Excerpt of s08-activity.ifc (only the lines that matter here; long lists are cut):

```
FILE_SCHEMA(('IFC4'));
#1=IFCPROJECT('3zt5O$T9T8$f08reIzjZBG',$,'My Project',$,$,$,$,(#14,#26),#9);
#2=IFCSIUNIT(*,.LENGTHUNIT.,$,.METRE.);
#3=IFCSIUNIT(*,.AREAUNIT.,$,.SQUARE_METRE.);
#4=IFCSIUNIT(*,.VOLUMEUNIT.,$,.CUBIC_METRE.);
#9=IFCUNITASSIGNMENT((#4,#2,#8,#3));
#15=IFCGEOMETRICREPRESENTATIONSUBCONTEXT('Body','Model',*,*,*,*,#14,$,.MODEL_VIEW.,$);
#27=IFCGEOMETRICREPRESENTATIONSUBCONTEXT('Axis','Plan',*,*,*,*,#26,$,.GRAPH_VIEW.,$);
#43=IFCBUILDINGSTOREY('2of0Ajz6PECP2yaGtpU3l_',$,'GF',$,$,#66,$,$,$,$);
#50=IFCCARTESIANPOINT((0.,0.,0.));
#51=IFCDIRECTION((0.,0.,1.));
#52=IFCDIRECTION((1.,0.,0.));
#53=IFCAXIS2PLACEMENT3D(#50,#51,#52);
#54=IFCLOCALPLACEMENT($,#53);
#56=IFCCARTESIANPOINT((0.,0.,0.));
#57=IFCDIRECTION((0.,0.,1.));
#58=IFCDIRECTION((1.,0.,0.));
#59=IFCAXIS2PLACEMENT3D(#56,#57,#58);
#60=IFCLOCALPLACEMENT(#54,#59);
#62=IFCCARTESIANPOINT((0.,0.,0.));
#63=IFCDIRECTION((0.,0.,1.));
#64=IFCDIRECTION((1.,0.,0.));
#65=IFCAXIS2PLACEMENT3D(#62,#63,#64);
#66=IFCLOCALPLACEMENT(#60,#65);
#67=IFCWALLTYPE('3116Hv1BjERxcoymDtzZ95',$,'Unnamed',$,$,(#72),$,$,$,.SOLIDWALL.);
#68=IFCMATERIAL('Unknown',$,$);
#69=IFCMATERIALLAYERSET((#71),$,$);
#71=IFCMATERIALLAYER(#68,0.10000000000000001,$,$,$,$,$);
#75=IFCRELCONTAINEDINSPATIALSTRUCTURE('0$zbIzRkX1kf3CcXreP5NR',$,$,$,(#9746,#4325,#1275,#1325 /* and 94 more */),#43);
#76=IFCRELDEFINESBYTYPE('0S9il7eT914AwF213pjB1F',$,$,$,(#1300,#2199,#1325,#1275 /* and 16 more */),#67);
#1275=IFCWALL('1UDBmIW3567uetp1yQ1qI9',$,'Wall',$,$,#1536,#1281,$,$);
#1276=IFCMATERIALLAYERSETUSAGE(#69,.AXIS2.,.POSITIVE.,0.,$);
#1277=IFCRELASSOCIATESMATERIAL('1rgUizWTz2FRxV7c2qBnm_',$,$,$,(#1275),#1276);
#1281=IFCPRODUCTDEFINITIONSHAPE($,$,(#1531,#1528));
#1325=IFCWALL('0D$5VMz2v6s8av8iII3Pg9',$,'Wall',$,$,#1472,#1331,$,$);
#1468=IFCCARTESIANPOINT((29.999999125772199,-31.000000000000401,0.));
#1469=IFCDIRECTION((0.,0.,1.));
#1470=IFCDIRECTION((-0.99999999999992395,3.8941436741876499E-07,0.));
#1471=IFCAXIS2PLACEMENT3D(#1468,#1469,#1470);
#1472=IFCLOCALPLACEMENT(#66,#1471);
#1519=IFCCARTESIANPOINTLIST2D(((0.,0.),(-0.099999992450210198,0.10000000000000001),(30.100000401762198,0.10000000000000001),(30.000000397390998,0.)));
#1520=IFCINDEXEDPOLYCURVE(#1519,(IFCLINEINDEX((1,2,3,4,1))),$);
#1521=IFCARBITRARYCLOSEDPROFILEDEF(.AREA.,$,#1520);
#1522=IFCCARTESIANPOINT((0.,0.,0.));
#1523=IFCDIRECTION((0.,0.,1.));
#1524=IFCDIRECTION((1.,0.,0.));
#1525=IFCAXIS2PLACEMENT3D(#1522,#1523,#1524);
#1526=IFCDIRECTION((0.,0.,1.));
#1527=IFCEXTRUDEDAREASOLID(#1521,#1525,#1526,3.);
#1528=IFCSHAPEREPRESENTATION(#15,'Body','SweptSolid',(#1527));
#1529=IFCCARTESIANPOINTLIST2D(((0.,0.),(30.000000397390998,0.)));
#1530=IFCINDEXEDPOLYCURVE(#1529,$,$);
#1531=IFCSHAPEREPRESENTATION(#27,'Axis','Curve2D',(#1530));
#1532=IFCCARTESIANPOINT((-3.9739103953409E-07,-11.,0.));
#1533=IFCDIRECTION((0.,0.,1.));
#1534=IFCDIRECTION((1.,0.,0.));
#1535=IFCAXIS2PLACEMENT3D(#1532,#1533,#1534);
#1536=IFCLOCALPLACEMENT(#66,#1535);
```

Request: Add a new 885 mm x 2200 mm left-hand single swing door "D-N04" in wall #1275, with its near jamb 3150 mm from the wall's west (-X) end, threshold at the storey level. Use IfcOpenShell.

```python
import numpy as np
import ifcopenshell
import ifcopenshell.api.feature
import ifcopenshell.api.geometry
import ifcopenshell.api.root
import ifcopenshell.api.spatial
import ifcopenshell.geom
import ifcopenshell.util.element
import ifcopenshell.util.placement
import ifcopenshell.util.representation
import ifcopenshell.util.shape
import ifcopenshell.util.unit

model = ifcopenshell.open("s08-activity.ifc")
unit_scale = ifcopenshell.util.unit.calculate_unit_scale(model)
settings = ifcopenshell.geom.settings()


def volume(element):
    """Net volume in cubic metres, openings subtracted."""
    shape = ifcopenshell.geom.create_shape(settings, element)
    return ifcopenshell.util.shape.get_volume(shape.geometry)


wall = model.by_guid("1UDBmIW3567uetp1yQ1qI9")
storey = ifcopenshell.util.element.get_container(wall, ifc_class="IfcBuildingStorey")
context = ifcopenshell.util.representation.get_context(model, "Model", "Body", "MODEL_VIEW")
before = volume(wall)

width, height, from_end, sill = 0.885, 2.2, 3.15, 0.0  # metres

# The wall runs along its own X axis, and the end named is its -X end.
wall_shape = ifcopenshell.geom.create_shape(settings, wall)
x, y, z = ifcopenshell.util.shape.get_vertices(wall_shape.geometry).T
start = x.min() + from_end
face, thickness = float(y.min()), float(y.max() - y.min())
wall_matrix = ifcopenshell.util.placement.get_local_placement(wall.ObjectPlacement)
level = ifcopenshell.util.placement.get_local_placement(storey.ObjectPlacement)[2, 3]


def in_wall(x, y):
    """Placement at x, y metres in the wall's axes, at sill height."""
    matrix = wall_matrix.copy()
    matrix[:, 3] = wall_matrix @ np.array([x / unit_scale, y / unit_scale, 0.0, 1.0])
    matrix[2, 3] = level + sill / unit_scale
    return matrix


# Opening: a box that overshoots both wall faces by 50 mm.
opening = ifcopenshell.api.root.create_entity(model, ifc_class="IfcOpeningElement", predefined_type="OPENING")
box = ifcopenshell.api.geometry.add_wall_representation(
    model, context=context, length=width, height=height, thickness=thickness + 0.1
)
ifcopenshell.api.geometry.assign_representation(model, product=opening, representation=box)
ifcopenshell.api.geometry.edit_object_placement(model, product=opening, matrix=in_wall(start, face - 0.05), is_si=False)
ifcopenshell.api.feature.add_feature(model, feature=opening, element=wall)

door = ifcopenshell.api.root.create_entity(model, ifc_class="IfcDoor", name="D-N04", predefined_type="DOOR")
door.OverallWidth, door.OverallHeight = width / unit_scale, height / unit_scale
door.OperationType = "SINGLE_SWING_LEFT"
body = ifcopenshell.api.geometry.add_door_representation(
    model,
    context=context,
    overall_width=door.OverallWidth,
    overall_height=door.OverallHeight,
    operation_type="SINGLE_SWING_LEFT",
    lining_properties={"LiningDepth": thickness / unit_scale, "ThresholdDepth": thickness / unit_scale},
)
ifcopenshell.api.geometry.assign_representation(model, product=door, representation=body)
ifcopenshell.api.spatial.assign_container(model, products=[door], relating_structure=storey)
ifcopenshell.api.feature.add_filling(model, opening=opening, element=door)

# The lining spans the wall, so the door starts at the wall face.
ifcopenshell.api.geometry.edit_object_placement(model, product=door, matrix=in_wall(start, face), is_si=False)

after = volume(wall)

print(f"wall volume {before:.3f} -> {after:.3f} m3")

model.write("s08-activity-out.ifc")
```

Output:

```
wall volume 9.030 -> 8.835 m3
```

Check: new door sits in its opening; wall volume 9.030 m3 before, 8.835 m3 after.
